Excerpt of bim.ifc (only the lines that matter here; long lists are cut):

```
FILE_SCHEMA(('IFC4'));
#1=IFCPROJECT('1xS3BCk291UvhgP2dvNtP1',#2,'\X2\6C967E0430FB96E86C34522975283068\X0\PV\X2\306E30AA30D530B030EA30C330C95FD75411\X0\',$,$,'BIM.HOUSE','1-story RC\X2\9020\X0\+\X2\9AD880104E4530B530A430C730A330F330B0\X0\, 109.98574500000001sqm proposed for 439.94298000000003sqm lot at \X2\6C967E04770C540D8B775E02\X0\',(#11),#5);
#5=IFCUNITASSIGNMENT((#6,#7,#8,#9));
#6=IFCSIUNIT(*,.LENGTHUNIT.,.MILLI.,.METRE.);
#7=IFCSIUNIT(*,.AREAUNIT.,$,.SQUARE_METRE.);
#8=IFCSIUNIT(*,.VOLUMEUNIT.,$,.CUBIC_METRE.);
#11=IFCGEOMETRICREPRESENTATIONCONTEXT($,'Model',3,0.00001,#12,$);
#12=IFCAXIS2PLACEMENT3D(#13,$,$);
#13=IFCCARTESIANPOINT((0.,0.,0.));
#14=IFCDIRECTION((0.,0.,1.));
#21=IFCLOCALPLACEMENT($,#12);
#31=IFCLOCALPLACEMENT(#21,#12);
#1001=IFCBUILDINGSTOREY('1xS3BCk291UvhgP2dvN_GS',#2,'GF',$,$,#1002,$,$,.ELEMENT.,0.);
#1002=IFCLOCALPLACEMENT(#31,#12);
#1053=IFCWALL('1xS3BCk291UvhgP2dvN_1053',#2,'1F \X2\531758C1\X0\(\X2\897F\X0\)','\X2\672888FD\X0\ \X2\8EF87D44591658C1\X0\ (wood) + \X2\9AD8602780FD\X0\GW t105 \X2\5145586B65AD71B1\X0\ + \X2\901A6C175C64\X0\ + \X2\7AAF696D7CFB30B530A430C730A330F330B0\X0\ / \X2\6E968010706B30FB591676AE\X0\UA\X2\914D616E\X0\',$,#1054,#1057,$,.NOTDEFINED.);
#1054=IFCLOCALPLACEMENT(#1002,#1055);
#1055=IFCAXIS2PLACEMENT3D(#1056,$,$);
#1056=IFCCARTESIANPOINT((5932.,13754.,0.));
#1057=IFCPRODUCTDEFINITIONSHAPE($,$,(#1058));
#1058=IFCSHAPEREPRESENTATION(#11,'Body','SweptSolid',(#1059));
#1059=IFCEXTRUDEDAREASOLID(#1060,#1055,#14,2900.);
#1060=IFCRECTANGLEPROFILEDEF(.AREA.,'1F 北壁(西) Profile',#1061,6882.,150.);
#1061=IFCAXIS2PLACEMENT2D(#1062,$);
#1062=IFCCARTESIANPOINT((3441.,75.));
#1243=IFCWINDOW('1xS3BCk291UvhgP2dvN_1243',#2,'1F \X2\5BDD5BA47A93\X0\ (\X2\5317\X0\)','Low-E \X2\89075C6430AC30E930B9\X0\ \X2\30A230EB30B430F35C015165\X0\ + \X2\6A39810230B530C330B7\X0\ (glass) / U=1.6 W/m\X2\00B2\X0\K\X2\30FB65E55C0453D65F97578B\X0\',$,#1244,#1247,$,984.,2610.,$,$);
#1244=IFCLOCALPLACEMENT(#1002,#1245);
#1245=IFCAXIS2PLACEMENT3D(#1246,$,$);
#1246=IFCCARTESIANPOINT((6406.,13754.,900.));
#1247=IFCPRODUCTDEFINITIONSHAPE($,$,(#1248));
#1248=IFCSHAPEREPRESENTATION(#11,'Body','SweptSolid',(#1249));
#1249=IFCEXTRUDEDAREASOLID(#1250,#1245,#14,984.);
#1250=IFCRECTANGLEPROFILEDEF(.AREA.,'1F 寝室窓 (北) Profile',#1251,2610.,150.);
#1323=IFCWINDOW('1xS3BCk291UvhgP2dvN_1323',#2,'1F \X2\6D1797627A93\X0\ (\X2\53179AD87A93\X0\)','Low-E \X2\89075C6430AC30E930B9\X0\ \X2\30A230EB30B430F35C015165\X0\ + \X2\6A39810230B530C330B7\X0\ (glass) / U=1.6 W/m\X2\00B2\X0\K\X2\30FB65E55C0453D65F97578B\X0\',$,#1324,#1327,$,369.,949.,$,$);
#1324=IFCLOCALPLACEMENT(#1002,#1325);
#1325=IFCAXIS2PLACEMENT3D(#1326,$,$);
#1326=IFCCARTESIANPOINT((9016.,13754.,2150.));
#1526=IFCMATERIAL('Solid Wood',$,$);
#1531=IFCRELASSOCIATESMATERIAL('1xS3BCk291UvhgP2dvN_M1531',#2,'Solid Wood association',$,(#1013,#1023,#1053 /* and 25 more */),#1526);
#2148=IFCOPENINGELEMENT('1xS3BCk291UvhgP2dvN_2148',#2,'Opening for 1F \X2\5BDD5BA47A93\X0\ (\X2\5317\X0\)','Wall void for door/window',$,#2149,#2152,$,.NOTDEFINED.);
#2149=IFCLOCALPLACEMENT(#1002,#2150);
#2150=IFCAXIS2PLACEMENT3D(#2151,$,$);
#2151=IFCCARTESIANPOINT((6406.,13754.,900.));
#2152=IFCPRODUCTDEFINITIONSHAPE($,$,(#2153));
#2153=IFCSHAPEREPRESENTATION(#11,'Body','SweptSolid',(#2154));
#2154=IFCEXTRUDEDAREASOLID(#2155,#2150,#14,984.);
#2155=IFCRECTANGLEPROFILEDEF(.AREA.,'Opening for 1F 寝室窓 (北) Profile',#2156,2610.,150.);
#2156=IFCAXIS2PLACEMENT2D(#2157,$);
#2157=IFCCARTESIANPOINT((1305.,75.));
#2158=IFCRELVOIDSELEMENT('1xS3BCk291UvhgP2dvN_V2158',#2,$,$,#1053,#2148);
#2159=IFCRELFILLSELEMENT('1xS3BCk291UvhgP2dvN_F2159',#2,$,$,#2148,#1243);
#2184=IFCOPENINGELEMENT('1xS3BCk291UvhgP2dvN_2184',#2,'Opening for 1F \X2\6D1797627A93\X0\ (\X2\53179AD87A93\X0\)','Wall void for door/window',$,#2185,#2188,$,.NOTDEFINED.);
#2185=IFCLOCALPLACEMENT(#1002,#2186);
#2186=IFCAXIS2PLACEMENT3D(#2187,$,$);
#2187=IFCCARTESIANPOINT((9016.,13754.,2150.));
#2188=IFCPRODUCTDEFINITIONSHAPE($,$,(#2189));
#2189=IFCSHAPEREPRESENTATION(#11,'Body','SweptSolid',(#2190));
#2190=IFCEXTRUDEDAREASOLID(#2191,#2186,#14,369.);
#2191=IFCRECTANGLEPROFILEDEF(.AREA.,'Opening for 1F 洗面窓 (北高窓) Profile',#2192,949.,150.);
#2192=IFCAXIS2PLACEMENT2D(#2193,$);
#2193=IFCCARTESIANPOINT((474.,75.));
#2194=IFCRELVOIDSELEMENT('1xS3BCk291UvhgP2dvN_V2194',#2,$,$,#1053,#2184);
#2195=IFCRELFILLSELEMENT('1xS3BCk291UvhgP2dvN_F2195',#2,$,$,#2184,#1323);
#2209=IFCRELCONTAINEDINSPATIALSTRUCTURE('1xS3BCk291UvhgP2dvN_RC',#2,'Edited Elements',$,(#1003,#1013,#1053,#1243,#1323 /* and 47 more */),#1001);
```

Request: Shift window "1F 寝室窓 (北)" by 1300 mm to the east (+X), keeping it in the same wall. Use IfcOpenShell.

```python
import ifcopenshell
import ifcopenshell.api.geometry
import ifcopenshell.util.placement

model = ifcopenshell.open("bim.ifc")

window = model.by_guid("1xS3BCk291UvhgP2dvN_1243")
opening = window.FillsVoids[0].RelatingOpeningElement
wall = opening.VoidsElements[0].RelatingBuildingElement

wall_matrix = ifcopenshell.util.placement.get_local_placement(wall.ObjectPlacement)
shift = wall_matrix[:3, 0] * 1300.0
before = ifcopenshell.util.placement.get_local_placement(window.ObjectPlacement)[:3, 3].copy()

# The window is not placed relative to its opening, so move both.
for product in (opening, window):
    matrix = ifcopenshell.util.placement.get_local_placement(product.ObjectPlacement)
    matrix[:3, 3] += shift
    ifcopenshell.api.geometry.edit_object_placement(model, product=product, matrix=matrix, is_si=False)

after = ifcopenshell.util.placement.get_local_placement(window.ObjectPlacement)[:3, 3]
print("window moved by", (after - before).round(3) + 0.0)

model.write("bim_updated.ifc")
```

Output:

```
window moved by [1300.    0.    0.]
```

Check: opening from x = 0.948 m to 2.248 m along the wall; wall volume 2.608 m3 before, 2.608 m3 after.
